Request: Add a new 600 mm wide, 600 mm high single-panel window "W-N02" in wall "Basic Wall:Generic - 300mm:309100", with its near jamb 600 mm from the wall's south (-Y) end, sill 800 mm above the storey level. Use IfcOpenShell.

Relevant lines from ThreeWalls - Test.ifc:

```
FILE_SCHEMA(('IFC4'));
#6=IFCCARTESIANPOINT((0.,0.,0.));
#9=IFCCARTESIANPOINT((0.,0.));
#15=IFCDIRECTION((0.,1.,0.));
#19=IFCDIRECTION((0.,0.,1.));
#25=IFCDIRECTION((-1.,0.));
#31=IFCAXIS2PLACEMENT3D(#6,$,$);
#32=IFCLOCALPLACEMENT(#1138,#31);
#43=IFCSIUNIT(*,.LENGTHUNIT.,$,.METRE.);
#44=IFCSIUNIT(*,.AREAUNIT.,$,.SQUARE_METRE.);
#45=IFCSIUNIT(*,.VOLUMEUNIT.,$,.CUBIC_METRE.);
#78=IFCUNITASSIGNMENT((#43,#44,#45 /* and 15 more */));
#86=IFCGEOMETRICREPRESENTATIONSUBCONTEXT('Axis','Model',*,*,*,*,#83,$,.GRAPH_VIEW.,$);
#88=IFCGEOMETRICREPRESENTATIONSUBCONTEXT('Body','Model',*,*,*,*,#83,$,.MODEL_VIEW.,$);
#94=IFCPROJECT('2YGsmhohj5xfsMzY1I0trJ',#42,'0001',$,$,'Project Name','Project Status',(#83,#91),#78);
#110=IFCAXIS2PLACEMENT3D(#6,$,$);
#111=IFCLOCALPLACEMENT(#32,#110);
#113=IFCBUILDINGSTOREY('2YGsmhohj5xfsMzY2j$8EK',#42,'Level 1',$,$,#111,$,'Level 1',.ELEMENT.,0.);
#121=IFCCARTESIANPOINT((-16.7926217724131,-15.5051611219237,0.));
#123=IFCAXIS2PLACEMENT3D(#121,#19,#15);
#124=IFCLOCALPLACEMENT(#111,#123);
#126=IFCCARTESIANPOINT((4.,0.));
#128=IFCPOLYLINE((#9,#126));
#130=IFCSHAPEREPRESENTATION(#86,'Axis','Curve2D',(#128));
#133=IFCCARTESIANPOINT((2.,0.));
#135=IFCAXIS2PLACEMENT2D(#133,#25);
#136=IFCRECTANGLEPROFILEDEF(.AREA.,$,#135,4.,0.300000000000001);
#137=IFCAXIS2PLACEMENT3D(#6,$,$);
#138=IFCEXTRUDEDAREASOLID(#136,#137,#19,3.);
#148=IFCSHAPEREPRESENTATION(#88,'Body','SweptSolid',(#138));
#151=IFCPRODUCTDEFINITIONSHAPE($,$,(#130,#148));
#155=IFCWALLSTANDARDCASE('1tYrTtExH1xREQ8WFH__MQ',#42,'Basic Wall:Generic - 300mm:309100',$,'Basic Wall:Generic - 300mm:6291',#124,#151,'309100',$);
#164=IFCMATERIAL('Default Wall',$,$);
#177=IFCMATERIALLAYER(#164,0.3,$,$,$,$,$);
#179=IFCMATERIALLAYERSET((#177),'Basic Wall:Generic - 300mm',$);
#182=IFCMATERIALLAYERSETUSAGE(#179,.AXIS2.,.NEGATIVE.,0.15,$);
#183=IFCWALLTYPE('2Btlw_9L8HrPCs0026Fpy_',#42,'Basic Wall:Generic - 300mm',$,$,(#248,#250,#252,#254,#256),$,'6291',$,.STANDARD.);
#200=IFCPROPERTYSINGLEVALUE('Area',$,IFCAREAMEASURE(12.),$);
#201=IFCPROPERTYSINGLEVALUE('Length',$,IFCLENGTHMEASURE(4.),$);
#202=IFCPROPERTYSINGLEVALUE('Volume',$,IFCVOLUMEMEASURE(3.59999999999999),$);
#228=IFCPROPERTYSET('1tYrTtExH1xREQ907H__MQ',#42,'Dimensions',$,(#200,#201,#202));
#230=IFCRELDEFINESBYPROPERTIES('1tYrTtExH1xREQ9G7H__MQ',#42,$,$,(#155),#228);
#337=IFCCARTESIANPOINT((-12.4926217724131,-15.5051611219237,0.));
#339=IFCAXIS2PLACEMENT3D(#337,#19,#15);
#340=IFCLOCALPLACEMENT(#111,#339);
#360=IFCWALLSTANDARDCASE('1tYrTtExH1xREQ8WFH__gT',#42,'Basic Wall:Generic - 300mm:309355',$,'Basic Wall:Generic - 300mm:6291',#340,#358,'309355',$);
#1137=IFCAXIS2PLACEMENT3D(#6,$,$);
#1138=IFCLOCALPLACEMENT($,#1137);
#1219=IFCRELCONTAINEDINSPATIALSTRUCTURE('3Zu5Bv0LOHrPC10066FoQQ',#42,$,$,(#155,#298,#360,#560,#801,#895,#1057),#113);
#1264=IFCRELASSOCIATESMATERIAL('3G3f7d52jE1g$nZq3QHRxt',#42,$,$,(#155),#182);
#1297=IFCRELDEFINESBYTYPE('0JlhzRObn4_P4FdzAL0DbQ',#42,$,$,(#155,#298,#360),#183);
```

```python
import numpy as np
import ifcopenshell
import ifcopenshell.api.feature
import ifcopenshell.api.geometry
import ifcopenshell.api.pset
import ifcopenshell.api.root
import ifcopenshell.api.spatial
import ifcopenshell.geom
import ifcopenshell.util.element
import ifcopenshell.util.placement
import ifcopenshell.util.representation
import ifcopenshell.util.shape
import ifcopenshell.util.unit

model = ifcopenshell.open("ThreeWalls - Test.ifc")
unit_scale = ifcopenshell.util.unit.calculate_unit_scale(model)
area_scale = ifcopenshell.util.unit.calculate_unit_scale(model, "AREAUNIT")
volume_scale = ifcopenshell.util.unit.calculate_unit_scale(model, "VOLUMEUNIT")
settings = ifcopenshell.geom.settings()


def volume(element):
    """Net volume in cubic metres, openings subtracted."""
    shape = ifcopenshell.geom.create_shape(settings, element)
    return ifcopenshell.util.shape.get_volume(shape.geometry)


wall = model.by_guid("1tYrTtExH1xREQ8WFH__MQ")
storey = ifcopenshell.util.element.get_container(wall, ifc_class="IfcBuildingStorey")
context = ifcopenshell.util.representation.get_context(model, "Model", "Body", "MODEL_VIEW")
before = volume(wall)

width, height, from_end, sill = 0.6, 0.6, 0.6, 0.8  # metres

# The wall runs along its own X axis, and the end named is its -X end.
wall_shape = ifcopenshell.geom.create_shape(settings, wall)
x, y, z = ifcopenshell.util.shape.get_vertices(wall_shape.geometry).T
start = x.min() + from_end
face, thickness = float(y.min()), float(y.max() - y.min())
wall_matrix = ifcopenshell.util.placement.get_local_placement(wall.ObjectPlacement)
level = ifcopenshell.util.placement.get_local_placement(storey.ObjectPlacement)[2, 3]


def in_wall(x, y):
    """Placement at x, y metres in the wall's axes, at sill height."""
    matrix = wall_matrix.copy()
    matrix[:, 3] = wall_matrix @ np.array([x / unit_scale, y / unit_scale, 0.0, 1.0])
    matrix[2, 3] = level + sill / unit_scale
    return matrix


# Opening: a box that overshoots both wall faces by 50 mm.
opening = ifcopenshell.api.root.create_entity(model, ifc_class="IfcOpeningElement", predefined_type="OPENING")
box = ifcopenshell.api.geometry.add_wall_representation(
    model, context=context, length=width, height=height, thickness=thickness + 0.1
)
ifcopenshell.api.geometry.assign_representation(model, product=opening, representation=box)
ifcopenshell.api.geometry.edit_object_placement(model, product=opening, matrix=in_wall(start, face - 0.05), is_si=False)
ifcopenshell.api.feature.add_feature(model, feature=opening, element=wall)

window = ifcopenshell.api.root.create_entity(model, ifc_class="IfcWindow", name="W-N02", predefined_type="WINDOW")
window.OverallWidth, window.OverallHeight = width / unit_scale, height / unit_scale
window.PartitioningType = "SINGLE_PANEL"
body = ifcopenshell.api.geometry.add_window_representation(
    model,
    context=context,
    overall_width=window.OverallWidth,
    overall_height=window.OverallHeight,
    partition_type="SINGLE_PANEL",
)
ifcopenshell.api.geometry.assign_representation(model, product=window, representation=body)
ifcopenshell.api.spatial.assign_container(model, products=[window], relating_structure=storey)
ifcopenshell.api.feature.add_filling(model, opening=opening, element=window)

# Centre the window in the wall's thickness.
ifcopenshell.api.geometry.edit_object_placement(model, product=window, matrix=in_wall(start, face), is_si=False)
window_shape = ifcopenshell.geom.create_shape(settings, window)
depth = ifcopenshell.util.shape.get_vertices(window_shape.geometry)[:, 1]
offset = face + thickness / 2 - (depth.min() + depth.max()) / 2
ifcopenshell.api.geometry.edit_object_placement(model, product=window, matrix=in_wall(start, offset), is_si=False)

after = volume(wall)

# Update the wall's stored quantities.
pset = model.by_id(ifcopenshell.util.element.get_pset(wall, "Dimensions", should_inherit=False)["id"])
ifcopenshell.api.pset.edit_pset(model, pset=pset, properties={
    "Area": model.create_entity("IfcAreaMeasure", after / thickness / area_scale),
    "Volume": model.create_entity("IfcVolumeMeasure", after / volume_scale),
})

print(f"wall volume {before:.3f} -> {after:.3f} m3")

model.write("ThreeWalls - Test_v2.ifc")
```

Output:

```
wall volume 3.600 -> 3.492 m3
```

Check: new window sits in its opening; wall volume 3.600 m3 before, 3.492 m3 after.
